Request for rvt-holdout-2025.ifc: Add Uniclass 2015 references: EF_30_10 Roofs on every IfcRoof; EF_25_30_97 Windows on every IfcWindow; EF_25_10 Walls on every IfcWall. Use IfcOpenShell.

First a look at what the model holds.

```python
import ifcopenshell

model = ifcopenshell.open("rvt-holdout-2025.ifc")
print(model.schema)
print("classifications:", [c.Name for c in model.by_type("IfcClassification")])
for ifc_class in ("IfcDoor", "IfcRoof", "IfcStair", "IfcWall", "IfcWindow"):
    print(ifc_class, len(model.by_type(ifc_class)))
```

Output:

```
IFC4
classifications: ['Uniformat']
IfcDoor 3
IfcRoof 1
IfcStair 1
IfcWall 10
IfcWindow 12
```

```python
import ifcopenshell
import ifcopenshell.api.classification

model = ifcopenshell.open("rvt-holdout-2025.ifc")

system = ifcopenshell.api.classification.add_classification(model, classification="Uniclass 2015")

codes = {
    "IfcRoof": ("EF_30_10", "Roofs"),
    "IfcWindow": ("EF_25_30_97", "Windows"),
    "IfcWall": ("EF_25_10", "Walls"),
}
for ifc_class, (code, name) in codes.items():
    products = model.by_type(ifc_class)
    ifcopenshell.api.classification.add_reference(
        model, products=products, classification=system, identification=code, name=name
    )
    print(code, len(products))

model.write("rvt-holdout-2025_updated.ifc")
```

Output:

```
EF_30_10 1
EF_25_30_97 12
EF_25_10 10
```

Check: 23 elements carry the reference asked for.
